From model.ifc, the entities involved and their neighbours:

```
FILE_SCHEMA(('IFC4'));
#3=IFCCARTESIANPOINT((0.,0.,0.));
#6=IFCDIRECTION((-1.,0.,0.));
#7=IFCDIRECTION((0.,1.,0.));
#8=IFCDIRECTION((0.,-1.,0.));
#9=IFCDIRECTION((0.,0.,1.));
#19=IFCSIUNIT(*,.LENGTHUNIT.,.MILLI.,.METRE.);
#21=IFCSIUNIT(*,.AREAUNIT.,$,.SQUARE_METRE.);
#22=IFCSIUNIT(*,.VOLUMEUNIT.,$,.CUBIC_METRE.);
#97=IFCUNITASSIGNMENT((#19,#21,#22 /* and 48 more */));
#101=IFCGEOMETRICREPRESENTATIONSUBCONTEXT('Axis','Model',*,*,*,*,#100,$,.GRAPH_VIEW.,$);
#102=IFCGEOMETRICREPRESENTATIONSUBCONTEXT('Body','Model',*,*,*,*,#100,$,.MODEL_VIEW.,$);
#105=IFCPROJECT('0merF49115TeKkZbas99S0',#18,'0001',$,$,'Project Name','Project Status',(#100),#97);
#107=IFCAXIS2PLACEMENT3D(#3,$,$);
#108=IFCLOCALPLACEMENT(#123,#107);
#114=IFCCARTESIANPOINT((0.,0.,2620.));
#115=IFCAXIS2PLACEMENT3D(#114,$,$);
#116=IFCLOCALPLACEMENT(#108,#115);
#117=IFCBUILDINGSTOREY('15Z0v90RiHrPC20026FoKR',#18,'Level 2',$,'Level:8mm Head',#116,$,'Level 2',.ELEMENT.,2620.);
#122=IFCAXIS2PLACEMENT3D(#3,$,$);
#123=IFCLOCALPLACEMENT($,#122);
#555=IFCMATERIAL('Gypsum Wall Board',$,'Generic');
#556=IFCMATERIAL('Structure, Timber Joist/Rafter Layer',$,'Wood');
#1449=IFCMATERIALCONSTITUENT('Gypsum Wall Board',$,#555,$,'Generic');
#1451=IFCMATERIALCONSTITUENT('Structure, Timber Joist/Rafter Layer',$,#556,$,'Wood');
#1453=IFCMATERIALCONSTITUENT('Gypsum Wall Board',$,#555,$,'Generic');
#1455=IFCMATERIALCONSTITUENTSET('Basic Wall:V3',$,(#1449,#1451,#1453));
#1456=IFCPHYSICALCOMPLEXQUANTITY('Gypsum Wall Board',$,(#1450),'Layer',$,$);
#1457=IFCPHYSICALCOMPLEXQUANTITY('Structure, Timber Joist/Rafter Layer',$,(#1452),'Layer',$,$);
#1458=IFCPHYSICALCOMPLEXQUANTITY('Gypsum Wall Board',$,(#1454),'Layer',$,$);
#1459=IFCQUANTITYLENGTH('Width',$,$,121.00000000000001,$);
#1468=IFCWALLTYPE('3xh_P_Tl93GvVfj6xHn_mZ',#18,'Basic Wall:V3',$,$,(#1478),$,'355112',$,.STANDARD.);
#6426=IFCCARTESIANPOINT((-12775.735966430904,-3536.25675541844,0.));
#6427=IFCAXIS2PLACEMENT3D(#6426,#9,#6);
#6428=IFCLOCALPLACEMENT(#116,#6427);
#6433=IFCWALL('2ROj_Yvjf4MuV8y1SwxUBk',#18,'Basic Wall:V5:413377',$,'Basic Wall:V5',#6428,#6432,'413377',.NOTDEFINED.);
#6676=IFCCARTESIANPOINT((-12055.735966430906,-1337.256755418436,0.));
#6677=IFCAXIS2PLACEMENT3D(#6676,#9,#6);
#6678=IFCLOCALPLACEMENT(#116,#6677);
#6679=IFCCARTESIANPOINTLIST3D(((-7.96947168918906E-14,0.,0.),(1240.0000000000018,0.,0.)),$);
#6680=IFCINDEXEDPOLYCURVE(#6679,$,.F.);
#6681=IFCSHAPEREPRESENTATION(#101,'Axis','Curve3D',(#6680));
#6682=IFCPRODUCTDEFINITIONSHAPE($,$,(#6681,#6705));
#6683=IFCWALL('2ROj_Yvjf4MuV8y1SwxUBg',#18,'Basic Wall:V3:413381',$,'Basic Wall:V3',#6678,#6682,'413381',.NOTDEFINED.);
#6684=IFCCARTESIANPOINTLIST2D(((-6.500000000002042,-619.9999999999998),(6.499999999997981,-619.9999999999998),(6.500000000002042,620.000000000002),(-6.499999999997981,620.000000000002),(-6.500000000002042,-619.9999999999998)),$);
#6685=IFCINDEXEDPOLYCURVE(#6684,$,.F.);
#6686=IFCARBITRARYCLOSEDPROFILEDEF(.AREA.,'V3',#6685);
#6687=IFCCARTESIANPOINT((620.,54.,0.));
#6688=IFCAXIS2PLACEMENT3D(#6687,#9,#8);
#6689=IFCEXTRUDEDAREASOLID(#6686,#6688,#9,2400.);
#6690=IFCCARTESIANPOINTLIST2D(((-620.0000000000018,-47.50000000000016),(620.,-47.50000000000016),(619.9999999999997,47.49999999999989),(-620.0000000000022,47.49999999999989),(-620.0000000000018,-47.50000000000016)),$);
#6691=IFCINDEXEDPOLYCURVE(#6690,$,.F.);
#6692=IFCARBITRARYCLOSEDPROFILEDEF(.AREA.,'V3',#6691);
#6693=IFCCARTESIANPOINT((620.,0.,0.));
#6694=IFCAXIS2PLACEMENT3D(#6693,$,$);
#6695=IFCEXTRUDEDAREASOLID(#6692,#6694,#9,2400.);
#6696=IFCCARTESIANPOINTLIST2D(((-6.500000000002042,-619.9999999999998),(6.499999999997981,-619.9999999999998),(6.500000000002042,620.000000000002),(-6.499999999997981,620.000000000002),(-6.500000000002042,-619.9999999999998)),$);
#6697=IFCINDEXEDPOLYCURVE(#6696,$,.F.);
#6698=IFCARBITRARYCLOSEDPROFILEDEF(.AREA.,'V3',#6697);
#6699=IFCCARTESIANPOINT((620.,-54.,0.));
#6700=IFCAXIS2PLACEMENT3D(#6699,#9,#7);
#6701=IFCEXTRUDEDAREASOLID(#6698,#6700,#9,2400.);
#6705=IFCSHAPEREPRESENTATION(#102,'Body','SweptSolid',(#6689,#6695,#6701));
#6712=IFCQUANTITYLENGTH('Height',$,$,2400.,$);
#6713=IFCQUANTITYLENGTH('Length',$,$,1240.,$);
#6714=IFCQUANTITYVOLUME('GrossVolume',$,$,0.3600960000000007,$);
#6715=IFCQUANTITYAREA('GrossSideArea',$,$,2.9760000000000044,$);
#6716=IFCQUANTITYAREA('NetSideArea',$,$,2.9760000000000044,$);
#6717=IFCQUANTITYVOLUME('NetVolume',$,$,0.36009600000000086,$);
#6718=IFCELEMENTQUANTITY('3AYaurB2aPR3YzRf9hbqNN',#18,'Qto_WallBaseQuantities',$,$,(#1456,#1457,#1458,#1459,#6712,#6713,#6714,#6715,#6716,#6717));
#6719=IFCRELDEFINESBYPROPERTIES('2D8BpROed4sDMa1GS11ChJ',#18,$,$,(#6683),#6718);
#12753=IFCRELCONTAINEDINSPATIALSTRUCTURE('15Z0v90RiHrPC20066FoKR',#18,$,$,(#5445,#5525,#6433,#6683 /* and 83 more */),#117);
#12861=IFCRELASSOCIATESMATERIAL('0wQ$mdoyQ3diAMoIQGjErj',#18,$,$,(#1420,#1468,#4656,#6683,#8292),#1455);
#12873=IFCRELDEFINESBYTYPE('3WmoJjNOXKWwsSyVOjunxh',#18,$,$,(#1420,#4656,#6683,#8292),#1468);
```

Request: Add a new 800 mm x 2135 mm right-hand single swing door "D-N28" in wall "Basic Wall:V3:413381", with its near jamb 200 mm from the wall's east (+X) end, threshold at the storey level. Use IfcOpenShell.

```python
import numpy as np
import ifcopenshell
import ifcopenshell.api.feature
import ifcopenshell.api.geometry
import ifcopenshell.api.pset
import ifcopenshell.api.root
import ifcopenshell.api.spatial
import ifcopenshell.geom
import ifcopenshell.util.element
import ifcopenshell.util.placement
import ifcopenshell.util.representation
import ifcopenshell.util.shape
import ifcopenshell.util.unit

model = ifcopenshell.open("model.ifc")
unit_scale = ifcopenshell.util.unit.calculate_unit_scale(model)
area_scale = ifcopenshell.util.unit.calculate_unit_scale(model, "AREAUNIT")
volume_scale = ifcopenshell.util.unit.calculate_unit_scale(model, "VOLUMEUNIT")
settings = ifcopenshell.geom.settings()


def volume(element):
    """Net volume in cubic metres, openings subtracted."""
    shape = ifcopenshell.geom.create_shape(settings, element)
    return ifcopenshell.util.shape.get_volume(shape.geometry)


wall = model.by_guid("2ROj_Yvjf4MuV8y1SwxUBg")
storey = ifcopenshell.util.element.get_container(wall, ifc_class="IfcBuildingStorey")
context = ifcopenshell.util.representation.get_context(model, "Model", "Body", "MODEL_VIEW")
before = volume(wall)

width, height, from_end, sill = 0.8, 2.135, 0.2, 0.0  # metres

# The wall runs along its own X axis, and the end named is its -X end.
wall_shape = ifcopenshell.geom.create_shape(settings, wall)
x, y, z = ifcopenshell.util.shape.get_vertices(wall_shape.geometry).T
start = x.min() + from_end
face, thickness = float(y.min()), float(y.max() - y.min())
wall_matrix = ifcopenshell.util.placement.get_local_placement(wall.ObjectPlacement)
level = ifcopenshell.util.placement.get_local_placement(storey.ObjectPlacement)[2, 3]


def in_wall(x, y):
    """Placement at x, y metres in the wall's axes, at sill height."""
    matrix = wall_matrix.copy()
    matrix[:, 3] = wall_matrix @ np.array([x / unit_scale, y / unit_scale, 0.0, 1.0])
    matrix[2, 3] = level + sill / unit_scale
    return matrix


# Opening: a box that overshoots both wall faces by 50 mm.
opening = ifcopenshell.api.root.create_entity(model, ifc_class="IfcOpeningElement", predefined_type="OPENING")
box = ifcopenshell.api.geometry.add_wall_representation(
    model, context=context, length=width, height=height, thickness=thickness + 0.1
)
ifcopenshell.api.geometry.assign_representation(model, product=opening, representation=box)
ifcopenshell.api.geometry.edit_object_placement(model, product=opening, matrix=in_wall(start, face - 0.05), is_si=False)
ifcopenshell.api.feature.add_feature(model, feature=opening, element=wall)

door = ifcopenshell.api.root.create_entity(model, ifc_class="IfcDoor", name="D-N28", predefined_type="DOOR")
door.OverallWidth, door.OverallHeight = width / unit_scale, height / unit_scale
door.OperationType = "SINGLE_SWING_RIGHT"
body = ifcopenshell.api.geometry.add_door_representation(
    model,
    context=context,
    overall_width=door.OverallWidth,
    overall_height=door.OverallHeight,
    operation_type="SINGLE_SWING_RIGHT",
    lining_properties={"LiningDepth": thickness / unit_scale, "ThresholdDepth": thickness / unit_scale},
)
ifcopenshell.api.geometry.assign_representation(model, product=door, representation=body)
ifcopenshell.api.spatial.assign_container(model, products=[door], relating_structure=storey)
ifcopenshell.api.feature.add_filling(model, opening=opening, element=door)

# The lining spans the wall, so the door starts at the wall face.
ifcopenshell.api.geometry.edit_object_placement(model, product=door, matrix=in_wall(start, face), is_si=False)

after = volume(wall)

# Update the wall's stored quantities.
qto = model.by_id(ifcopenshell.util.element.get_pset(wall, "Qto_WallBaseQuantities", should_inherit=False)["id"])
ifcopenshell.api.pset.edit_qto(model, qto=qto, properties={
    "NetSideArea": after / thickness / area_scale,
    "NetVolume": after / volume_scale,
})

print(f"wall volume {before:.3f} -> {after:.3f} m3")

model.write("model-out.ifc")
```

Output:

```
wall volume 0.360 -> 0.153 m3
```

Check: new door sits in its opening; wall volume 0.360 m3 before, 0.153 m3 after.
